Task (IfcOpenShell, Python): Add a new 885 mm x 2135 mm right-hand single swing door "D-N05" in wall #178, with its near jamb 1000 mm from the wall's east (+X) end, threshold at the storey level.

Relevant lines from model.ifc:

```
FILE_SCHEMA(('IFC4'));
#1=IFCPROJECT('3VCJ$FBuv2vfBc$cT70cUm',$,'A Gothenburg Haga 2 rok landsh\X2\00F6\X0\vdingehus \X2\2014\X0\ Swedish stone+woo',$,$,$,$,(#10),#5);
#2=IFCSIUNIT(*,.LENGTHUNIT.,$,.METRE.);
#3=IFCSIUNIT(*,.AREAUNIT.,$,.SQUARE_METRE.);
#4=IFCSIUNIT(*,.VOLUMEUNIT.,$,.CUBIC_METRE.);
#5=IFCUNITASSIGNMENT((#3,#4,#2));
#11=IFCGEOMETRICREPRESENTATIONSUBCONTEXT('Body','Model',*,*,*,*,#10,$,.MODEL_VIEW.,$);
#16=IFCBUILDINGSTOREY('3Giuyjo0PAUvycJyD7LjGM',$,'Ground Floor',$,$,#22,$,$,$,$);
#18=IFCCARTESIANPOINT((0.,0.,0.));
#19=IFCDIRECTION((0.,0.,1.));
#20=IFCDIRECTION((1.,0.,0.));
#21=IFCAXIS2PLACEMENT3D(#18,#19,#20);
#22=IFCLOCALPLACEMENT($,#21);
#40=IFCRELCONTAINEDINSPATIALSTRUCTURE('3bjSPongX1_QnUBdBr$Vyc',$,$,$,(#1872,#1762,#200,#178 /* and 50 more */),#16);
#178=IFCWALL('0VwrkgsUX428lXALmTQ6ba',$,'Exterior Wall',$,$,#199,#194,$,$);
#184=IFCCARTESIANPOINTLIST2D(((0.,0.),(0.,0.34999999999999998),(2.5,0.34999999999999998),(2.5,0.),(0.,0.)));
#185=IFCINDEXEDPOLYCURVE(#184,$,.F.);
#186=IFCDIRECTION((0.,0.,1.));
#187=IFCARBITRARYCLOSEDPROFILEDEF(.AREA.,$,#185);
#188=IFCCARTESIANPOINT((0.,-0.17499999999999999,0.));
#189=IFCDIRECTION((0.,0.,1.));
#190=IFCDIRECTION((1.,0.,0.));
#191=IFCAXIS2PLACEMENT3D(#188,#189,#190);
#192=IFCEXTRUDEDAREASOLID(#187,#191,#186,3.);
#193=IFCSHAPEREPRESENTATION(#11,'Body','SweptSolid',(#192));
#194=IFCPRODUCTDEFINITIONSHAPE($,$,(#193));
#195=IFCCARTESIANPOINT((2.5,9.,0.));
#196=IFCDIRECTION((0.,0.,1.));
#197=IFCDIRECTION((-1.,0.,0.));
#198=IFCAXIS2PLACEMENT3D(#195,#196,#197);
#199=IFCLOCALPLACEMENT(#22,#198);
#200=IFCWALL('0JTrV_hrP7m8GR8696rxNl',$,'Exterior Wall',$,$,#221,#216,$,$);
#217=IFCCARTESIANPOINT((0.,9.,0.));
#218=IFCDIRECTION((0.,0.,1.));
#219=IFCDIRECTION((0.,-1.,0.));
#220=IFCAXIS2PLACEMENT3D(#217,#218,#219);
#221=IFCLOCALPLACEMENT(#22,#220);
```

```python
import numpy as np
import ifcopenshell
import ifcopenshell.api.feature
import ifcopenshell.api.geometry
import ifcopenshell.api.root
import ifcopenshell.api.spatial
import ifcopenshell.geom
import ifcopenshell.util.element
import ifcopenshell.util.placement
import ifcopenshell.util.representation
import ifcopenshell.util.shape
import ifcopenshell.util.unit

model = ifcopenshell.open("model.ifc")
unit_scale = ifcopenshell.util.unit.calculate_unit_scale(model)
settings = ifcopenshell.geom.settings()


def volume(element):
    """Net volume in cubic metres, openings subtracted."""
    shape = ifcopenshell.geom.create_shape(settings, element)
    return ifcopenshell.util.shape.get_volume(shape.geometry)


wall = model.by_id(178)
storey = ifcopenshell.util.element.get_container(wall, ifc_class="IfcBuildingStorey")
context = ifcopenshell.util.representation.get_context(model, "Model", "Body", "MODEL_VIEW")
before = volume(wall)

width, height, from_end, sill = 0.885, 2.135, 1, 0.0  # metres

# The wall runs along its own X axis, and the end named is its -X end.
wall_shape = ifcopenshell.geom.create_shape(settings, wall)
x, y, z = ifcopenshell.util.shape.get_vertices(wall_shape.geometry).T
start = x.min() + from_end
face, thickness = float(y.min()), float(y.max() - y.min())
wall_matrix = ifcopenshell.util.placement.get_local_placement(wall.ObjectPlacement)
level = ifcopenshell.util.placement.get_local_placement(storey.ObjectPlacement)[2, 3]


def in_wall(x, y):
    """Placement at x, y metres in the wall's axes, at sill height."""
    matrix = wall_matrix.copy()
    matrix[:, 3] = wall_matrix @ np.array([x / unit_scale, y / unit_scale, 0.0, 1.0])
    matrix[2, 3] = level + sill / unit_scale
    return matrix


# Opening: a box that overshoots both wall faces by 50 mm.
opening = ifcopenshell.api.root.create_entity(model, ifc_class="IfcOpeningElement", predefined_type="OPENING")
box = ifcopenshell.api.geometry.add_wall_representation(
    model, context=context, length=width, height=height, thickness=thickness + 0.1
)
ifcopenshell.api.geometry.assign_representation(model, product=opening, representation=box)
ifcopenshell.api.geometry.edit_object_placement(model, product=opening, matrix=in_wall(start, face - 0.05), is_si=False)
ifcopenshell.api.feature.add_feature(model, feature=opening, element=wall)

door = ifcopenshell.api.root.create_entity(model, ifc_class="IfcDoor", name="D-N05", predefined_type="DOOR")
door.OverallWidth, door.OverallHeight = width / unit_scale, height / unit_scale
door.OperationType = "SINGLE_SWING_RIGHT"
body = ifcopenshell.api.geometry.add_door_representation(
    model,
    context=context,
    overall_width=door.OverallWidth,
    overall_height=door.OverallHeight,
    operation_type="SINGLE_SWING_RIGHT",
    lining_properties={"LiningDepth": thickness / unit_scale, "ThresholdDepth": thickness / unit_scale},
)
ifcopenshell.api.geometry.assign_representation(model, product=door, representation=body)
ifcopenshell.api.spatial.assign_container(model, products=[door], relating_structure=storey)
ifcopenshell.api.feature.add_filling(model, opening=opening, element=door)

# The lining spans the wall, so the door starts at the wall face.
ifcopenshell.api.geometry.edit_object_placement(model, product=door, matrix=in_wall(start, face), is_si=False)

after = volume(wall)

print(f"wall volume {before:.3f} -> {after:.3f} m3")

model.write("model_edited.ifc")
```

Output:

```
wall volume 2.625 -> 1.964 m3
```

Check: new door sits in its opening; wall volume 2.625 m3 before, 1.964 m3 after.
